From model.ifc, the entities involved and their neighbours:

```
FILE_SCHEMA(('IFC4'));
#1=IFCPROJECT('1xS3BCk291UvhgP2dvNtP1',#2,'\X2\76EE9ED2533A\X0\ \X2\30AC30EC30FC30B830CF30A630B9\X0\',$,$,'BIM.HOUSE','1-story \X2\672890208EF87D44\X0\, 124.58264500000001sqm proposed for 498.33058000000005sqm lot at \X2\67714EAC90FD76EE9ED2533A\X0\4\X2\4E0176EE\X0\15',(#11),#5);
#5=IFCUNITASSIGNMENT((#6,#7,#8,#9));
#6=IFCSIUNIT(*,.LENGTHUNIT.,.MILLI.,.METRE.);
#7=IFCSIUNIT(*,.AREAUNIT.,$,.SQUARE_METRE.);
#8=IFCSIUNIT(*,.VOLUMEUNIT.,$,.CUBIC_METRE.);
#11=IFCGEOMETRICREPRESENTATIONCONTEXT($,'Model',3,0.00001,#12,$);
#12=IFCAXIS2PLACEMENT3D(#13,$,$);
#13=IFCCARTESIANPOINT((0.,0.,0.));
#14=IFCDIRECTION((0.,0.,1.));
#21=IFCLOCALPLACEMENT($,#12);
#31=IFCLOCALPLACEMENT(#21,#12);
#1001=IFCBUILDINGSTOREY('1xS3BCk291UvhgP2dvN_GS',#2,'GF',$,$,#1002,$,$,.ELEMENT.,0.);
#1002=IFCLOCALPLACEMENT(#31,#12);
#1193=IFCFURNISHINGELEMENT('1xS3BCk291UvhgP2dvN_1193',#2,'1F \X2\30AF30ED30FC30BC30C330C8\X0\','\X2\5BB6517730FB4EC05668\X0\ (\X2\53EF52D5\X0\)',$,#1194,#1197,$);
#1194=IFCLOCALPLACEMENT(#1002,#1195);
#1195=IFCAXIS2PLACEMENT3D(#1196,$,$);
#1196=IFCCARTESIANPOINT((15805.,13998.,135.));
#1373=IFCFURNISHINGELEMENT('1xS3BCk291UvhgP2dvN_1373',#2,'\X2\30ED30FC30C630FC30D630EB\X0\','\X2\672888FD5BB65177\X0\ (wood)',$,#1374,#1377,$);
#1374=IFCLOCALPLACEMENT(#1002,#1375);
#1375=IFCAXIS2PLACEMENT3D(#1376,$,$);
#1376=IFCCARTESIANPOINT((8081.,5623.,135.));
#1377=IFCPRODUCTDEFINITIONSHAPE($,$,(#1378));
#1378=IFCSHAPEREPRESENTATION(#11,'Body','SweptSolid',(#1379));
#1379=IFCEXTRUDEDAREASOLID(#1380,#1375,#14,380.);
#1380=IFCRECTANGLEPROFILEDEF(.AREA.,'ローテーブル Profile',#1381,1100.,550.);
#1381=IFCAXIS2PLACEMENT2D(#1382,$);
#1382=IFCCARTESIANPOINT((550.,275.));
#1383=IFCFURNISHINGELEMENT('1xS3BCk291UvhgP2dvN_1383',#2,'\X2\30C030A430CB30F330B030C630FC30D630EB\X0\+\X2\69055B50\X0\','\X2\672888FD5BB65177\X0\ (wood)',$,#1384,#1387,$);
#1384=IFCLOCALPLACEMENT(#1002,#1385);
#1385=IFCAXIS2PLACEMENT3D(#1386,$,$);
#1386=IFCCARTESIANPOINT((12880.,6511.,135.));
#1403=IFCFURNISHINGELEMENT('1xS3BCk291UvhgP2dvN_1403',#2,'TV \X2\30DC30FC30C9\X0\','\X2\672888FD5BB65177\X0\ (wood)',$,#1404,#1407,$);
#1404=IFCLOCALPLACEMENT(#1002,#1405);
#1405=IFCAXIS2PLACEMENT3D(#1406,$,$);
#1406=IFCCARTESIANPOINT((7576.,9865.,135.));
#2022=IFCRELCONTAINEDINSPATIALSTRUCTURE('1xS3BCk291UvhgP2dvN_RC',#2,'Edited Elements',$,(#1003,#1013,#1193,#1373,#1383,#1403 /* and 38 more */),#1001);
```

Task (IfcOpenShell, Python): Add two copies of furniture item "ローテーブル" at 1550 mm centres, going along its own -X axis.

```python
import ifcopenshell
import ifcopenshell.api.geometry
import ifcopenshell.api.root
import ifcopenshell.util.element
import ifcopenshell.util.placement

model = ifcopenshell.open("model.ifc")


def reuse_history(source, copy):
    """copy_class also copies each property set's owner history, people and application; keep the originals."""
    for rel in copy.IsDefinedBy:
        if rel.is_a("IfcRelDefinesByProperties") and (history := rel.RelatingPropertyDefinition.OwnerHistory):
            rel.RelatingPropertyDefinition.OwnerHistory = source.OwnerHistory
            ifcopenshell.util.element.remove_deep2(model, history)


source = model.by_guid("1xS3BCk291UvhgP2dvN_1373")
base = ifcopenshell.util.placement.get_local_placement(source.ObjectPlacement)
step = -base[:3, 0] * 1550.0

for i in range(1, 3):
    copy = ifcopenshell.api.root.copy_class(model, product=source)
    copy.Representation = ifcopenshell.util.element.copy_deep(
        model, source.Representation, exclude=["IfcGeometricRepresentationContext", "IfcRepresentationMap"]
    )
    reuse_history(source, copy)
    matrix = base.copy()
    matrix[:3, 3] += i * step
    print("added at", matrix[:3, 3].round(3) + 0.0)
    ifcopenshell.api.geometry.edit_object_placement(model, product=copy, matrix=matrix, is_si=False)

model.write("model_v2.ifc")
```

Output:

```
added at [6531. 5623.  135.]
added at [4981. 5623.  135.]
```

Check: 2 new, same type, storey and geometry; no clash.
